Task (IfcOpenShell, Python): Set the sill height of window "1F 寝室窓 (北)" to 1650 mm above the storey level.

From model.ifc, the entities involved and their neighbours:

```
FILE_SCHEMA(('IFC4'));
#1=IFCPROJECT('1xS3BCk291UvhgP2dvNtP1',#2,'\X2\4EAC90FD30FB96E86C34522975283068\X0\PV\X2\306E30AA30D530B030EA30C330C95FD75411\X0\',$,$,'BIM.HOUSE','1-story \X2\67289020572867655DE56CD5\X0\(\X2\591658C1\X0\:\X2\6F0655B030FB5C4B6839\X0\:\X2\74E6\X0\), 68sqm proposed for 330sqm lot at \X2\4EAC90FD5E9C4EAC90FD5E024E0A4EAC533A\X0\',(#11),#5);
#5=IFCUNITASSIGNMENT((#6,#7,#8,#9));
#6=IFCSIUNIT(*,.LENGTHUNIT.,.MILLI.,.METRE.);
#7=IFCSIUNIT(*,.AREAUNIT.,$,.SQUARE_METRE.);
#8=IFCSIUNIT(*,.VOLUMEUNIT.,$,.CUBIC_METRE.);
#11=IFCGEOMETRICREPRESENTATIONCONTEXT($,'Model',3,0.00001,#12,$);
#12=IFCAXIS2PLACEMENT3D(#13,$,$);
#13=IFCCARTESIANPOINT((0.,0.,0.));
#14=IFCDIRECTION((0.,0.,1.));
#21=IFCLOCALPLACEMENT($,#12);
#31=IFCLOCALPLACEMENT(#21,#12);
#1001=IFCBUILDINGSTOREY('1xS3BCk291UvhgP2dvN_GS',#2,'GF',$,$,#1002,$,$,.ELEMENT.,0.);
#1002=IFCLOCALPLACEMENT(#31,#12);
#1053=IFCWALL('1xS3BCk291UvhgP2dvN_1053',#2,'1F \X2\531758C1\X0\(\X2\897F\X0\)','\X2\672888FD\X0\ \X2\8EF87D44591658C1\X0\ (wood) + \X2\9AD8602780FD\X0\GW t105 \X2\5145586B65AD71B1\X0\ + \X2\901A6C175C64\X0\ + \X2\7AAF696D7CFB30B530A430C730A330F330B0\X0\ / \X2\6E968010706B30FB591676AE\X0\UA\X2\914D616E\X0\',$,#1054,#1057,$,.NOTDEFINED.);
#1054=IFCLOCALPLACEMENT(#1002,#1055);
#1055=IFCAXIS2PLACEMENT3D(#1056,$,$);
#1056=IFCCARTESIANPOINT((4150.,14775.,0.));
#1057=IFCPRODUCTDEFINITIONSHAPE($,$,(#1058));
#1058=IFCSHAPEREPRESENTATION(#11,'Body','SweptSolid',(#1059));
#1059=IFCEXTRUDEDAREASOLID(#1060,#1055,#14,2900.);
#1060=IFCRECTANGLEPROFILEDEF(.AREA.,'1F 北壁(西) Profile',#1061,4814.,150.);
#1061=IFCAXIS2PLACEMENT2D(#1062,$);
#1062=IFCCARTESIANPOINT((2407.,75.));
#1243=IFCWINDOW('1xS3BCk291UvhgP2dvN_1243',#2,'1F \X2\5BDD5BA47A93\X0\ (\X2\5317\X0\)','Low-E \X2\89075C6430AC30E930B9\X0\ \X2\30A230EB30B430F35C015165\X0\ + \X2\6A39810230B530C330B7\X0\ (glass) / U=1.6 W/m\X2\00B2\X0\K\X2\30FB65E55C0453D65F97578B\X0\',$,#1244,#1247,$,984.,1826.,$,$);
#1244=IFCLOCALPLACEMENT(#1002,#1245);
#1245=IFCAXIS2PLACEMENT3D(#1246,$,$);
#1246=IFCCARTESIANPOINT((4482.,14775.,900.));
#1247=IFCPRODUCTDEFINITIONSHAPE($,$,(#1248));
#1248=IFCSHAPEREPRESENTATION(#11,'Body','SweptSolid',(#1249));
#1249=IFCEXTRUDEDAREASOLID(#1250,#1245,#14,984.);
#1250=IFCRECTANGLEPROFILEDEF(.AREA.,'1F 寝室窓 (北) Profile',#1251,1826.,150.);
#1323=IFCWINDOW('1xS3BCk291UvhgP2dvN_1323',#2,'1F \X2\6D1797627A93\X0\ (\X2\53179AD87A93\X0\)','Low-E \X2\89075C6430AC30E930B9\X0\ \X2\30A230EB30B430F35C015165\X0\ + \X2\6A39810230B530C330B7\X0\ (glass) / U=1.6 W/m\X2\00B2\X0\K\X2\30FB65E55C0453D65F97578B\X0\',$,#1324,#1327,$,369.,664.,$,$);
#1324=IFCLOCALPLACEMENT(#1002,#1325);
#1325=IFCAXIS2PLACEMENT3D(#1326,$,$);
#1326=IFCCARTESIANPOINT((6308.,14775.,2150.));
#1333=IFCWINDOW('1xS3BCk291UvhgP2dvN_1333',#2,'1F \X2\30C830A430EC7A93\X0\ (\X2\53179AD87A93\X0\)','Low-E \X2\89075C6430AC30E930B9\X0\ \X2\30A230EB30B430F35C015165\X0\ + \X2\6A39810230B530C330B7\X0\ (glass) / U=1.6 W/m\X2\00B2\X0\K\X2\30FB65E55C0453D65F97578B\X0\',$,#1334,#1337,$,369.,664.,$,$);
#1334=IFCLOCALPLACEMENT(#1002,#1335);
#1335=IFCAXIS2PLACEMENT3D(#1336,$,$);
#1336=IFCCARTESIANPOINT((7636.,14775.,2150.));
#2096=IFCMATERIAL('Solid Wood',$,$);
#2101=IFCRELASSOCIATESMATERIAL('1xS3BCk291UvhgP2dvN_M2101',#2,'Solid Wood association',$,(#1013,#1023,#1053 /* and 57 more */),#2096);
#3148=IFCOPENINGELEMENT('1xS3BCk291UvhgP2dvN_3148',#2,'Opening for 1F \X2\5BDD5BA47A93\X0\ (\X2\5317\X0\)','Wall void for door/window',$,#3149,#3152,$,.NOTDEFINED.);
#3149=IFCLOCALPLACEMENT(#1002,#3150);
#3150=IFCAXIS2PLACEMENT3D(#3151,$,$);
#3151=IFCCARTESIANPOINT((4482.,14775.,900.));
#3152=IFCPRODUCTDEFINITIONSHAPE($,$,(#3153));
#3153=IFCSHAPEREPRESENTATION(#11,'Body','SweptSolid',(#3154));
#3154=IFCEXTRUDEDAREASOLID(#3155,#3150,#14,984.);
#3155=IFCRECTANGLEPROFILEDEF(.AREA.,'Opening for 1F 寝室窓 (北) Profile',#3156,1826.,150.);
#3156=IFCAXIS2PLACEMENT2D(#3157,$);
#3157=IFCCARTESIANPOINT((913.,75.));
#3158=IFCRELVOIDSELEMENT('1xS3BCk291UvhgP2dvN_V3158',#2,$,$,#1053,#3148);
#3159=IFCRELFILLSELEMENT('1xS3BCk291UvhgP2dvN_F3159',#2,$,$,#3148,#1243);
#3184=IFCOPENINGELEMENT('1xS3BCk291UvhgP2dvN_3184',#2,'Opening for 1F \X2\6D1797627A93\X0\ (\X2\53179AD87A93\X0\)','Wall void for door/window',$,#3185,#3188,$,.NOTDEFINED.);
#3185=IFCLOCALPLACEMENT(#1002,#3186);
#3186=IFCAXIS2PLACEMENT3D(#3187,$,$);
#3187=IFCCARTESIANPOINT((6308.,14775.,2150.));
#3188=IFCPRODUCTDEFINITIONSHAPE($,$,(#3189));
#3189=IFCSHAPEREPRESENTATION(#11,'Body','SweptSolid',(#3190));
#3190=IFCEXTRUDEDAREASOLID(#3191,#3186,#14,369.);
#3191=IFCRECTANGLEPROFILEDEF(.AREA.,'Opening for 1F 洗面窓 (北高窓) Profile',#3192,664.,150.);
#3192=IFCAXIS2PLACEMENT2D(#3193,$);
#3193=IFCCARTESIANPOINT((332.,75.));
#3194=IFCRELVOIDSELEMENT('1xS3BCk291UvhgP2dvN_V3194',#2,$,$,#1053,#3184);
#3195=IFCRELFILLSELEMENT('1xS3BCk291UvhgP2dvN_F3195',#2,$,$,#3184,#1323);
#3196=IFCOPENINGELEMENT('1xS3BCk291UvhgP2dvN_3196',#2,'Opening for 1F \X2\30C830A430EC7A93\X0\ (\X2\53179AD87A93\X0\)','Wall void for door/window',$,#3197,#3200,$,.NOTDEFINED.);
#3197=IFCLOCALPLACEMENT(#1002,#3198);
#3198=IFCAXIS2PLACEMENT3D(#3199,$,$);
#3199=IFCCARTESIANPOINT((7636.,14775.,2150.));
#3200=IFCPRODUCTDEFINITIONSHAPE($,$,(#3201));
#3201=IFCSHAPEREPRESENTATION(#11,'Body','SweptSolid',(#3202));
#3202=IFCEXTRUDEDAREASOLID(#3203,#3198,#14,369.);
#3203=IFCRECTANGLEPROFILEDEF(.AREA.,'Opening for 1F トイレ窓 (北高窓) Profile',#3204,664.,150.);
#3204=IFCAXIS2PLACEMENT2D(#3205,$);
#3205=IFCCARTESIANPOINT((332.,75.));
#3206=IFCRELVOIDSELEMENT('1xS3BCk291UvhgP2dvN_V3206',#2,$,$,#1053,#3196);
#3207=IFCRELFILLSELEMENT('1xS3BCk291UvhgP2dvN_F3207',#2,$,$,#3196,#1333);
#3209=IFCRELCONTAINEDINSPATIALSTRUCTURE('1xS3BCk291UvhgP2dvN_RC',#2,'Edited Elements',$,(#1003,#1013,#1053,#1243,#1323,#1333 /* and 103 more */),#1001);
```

```python
import numpy as np
import ifcopenshell
import ifcopenshell.api.geometry
import ifcopenshell.geom
import ifcopenshell.util.element
import ifcopenshell.util.placement
import ifcopenshell.util.shape
import ifcopenshell.util.unit

model = ifcopenshell.open("model.ifc")
unit_scale = ifcopenshell.util.unit.calculate_unit_scale(model)

window = model.by_id(1243)
opening = window.FillsVoids[0].RelatingOpeningElement
storey = ifcopenshell.util.element.get_container(window, ifc_class="IfcBuildingStorey")
level = ifcopenshell.util.placement.get_local_placement(storey.ObjectPlacement)[2, 3]

# The opening's origin need not be at the sill, so measure its lowest point.
shape = ifcopenshell.geom.create_shape(ifcopenshell.geom.settings(), opening)
bottom = ifcopenshell.util.shape.get_shape_bottom_elevation(shape, shape.geometry) / unit_scale
dz = level + 1.65 / unit_scale - bottom

shift = np.array([0.0, 0.0, dz])
# The window is not placed relative to its opening, so move both.
for product in (opening, window):
    matrix = ifcopenshell.util.placement.get_local_placement(product.ObjectPlacement)
    matrix[:3, 3] += shift
    ifcopenshell.api.geometry.edit_object_placement(model, product=product, matrix=matrix, is_si=False)

print(f"moved by {dz * unit_scale:+.3f} m")

model.write("model_updated.ifc")
```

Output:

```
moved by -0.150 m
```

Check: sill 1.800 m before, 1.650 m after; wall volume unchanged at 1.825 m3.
